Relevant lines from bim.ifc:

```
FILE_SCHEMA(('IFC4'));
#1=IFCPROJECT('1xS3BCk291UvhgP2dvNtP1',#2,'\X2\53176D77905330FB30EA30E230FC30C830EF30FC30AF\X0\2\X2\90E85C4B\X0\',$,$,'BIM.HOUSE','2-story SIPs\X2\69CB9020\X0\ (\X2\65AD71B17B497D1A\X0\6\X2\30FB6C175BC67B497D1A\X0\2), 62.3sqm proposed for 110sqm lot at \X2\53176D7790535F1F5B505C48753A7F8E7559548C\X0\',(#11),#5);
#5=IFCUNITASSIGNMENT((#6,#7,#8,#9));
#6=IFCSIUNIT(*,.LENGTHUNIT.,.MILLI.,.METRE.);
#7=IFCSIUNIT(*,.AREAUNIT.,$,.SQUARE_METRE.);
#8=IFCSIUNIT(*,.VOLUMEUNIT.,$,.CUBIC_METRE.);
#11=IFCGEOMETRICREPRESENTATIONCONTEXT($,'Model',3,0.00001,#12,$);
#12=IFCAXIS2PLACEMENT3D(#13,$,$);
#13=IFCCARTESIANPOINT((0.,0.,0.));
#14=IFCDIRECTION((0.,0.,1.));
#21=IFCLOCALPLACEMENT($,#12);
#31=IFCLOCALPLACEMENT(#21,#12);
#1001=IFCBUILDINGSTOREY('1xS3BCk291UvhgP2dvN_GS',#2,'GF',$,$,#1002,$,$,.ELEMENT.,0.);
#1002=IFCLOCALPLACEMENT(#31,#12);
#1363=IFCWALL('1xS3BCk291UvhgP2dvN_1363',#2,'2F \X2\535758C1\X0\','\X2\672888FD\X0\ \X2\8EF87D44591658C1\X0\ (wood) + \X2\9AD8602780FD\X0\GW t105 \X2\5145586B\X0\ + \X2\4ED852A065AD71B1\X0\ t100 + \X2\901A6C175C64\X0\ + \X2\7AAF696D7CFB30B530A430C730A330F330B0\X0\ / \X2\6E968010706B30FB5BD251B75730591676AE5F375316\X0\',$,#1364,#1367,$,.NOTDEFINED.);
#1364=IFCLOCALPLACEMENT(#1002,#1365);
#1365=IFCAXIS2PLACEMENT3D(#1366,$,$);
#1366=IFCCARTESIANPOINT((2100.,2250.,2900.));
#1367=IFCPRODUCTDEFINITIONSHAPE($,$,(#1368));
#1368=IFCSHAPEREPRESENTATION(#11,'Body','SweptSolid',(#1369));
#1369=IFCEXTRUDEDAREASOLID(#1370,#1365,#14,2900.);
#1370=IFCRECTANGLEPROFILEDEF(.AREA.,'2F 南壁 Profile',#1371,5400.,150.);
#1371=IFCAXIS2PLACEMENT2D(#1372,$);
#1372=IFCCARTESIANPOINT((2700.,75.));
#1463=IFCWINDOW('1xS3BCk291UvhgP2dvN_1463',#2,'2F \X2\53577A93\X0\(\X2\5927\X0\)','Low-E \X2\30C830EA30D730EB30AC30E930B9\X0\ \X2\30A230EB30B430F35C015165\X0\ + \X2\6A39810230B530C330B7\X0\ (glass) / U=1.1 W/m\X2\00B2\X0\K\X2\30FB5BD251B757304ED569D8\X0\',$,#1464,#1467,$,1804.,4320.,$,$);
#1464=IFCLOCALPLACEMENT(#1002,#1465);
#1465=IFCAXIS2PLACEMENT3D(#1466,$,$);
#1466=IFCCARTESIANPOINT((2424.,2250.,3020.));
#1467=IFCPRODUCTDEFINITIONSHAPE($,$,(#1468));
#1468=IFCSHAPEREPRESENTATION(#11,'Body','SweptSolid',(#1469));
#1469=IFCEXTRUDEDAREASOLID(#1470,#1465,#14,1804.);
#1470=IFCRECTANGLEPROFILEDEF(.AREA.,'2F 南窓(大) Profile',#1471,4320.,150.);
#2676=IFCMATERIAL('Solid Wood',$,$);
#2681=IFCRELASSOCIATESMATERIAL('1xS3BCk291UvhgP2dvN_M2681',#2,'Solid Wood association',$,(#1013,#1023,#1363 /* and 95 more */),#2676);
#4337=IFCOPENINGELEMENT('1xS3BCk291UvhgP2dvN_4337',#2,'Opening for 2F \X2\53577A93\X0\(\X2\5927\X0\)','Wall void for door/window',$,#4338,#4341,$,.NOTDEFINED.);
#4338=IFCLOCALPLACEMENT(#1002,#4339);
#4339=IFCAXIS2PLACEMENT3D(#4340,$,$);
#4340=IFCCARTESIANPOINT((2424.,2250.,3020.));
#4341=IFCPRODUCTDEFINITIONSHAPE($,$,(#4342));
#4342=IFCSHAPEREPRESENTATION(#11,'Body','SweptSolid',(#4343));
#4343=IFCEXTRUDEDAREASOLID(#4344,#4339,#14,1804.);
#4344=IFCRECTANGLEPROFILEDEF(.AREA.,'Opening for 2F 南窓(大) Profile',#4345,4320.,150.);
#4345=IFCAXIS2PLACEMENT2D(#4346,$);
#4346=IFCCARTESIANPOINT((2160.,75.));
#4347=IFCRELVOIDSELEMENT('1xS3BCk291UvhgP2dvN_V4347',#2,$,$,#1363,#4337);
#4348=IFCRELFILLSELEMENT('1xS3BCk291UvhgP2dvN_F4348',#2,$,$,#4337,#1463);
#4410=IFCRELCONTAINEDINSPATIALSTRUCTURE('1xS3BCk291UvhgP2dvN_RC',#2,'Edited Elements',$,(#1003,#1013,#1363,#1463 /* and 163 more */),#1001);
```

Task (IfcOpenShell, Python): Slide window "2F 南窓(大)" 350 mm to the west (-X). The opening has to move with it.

```python
import ifcopenshell
import ifcopenshell.api.geometry
import ifcopenshell.util.placement
import ifcopenshell.util.unit

model = ifcopenshell.open("bim.ifc")
unit_scale = ifcopenshell.util.unit.calculate_unit_scale(model)

window = model.by_guid("1xS3BCk291UvhgP2dvN_1463")
opening = window.FillsVoids[0].RelatingOpeningElement
wall = opening.VoidsElements[0].RelatingBuildingElement

wall_matrix = ifcopenshell.util.placement.get_local_placement(wall.ObjectPlacement)
shift = wall_matrix[:3, 0] * -0.35 / unit_scale
before = ifcopenshell.util.placement.get_local_placement(window.ObjectPlacement)[:3, 3].copy()

# The window is not placed relative to its opening, so move both.
for product in (opening, window):
    matrix = ifcopenshell.util.placement.get_local_placement(product.ObjectPlacement)
    matrix[:3, 3] += shift
    ifcopenshell.api.geometry.edit_object_placement(model, product=product, matrix=matrix, is_si=False)

after = ifcopenshell.util.placement.get_local_placement(window.ObjectPlacement)[:3, 3]
print("window moved by", (after - before).round(3) + 0.0)

model.write("bim_updated.ifc")
```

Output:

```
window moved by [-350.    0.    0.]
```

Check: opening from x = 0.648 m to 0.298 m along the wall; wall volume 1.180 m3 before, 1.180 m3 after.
